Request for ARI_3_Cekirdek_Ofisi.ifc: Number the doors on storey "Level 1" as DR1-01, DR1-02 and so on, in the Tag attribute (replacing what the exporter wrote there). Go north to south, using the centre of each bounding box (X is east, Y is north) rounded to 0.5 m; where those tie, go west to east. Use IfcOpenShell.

First a look at what the model holds.

```python
import ifcopenshell
import ifcopenshell.util.element
import ifcopenshell.util.placement

model = ifcopenshell.open("ARI_3_Cekirdek_Ofisi.ifc")
print(model.schema)
storey = next(s for s in model.by_type("IfcBuildingStorey") if s.Name == "Level 1")
doors = [e for e in ifcopenshell.util.element.get_decomposition(storey) if e.is_a("IfcDoor")]
for e in sorted(doors, key=lambda e: e.id()):
    origin = ifcopenshell.util.placement.get_local_placement(e.ObjectPlacement)[:3, 3]
    print(e.id(), e.Tag, e.Name, origin.round(2) + 0.0, sep=" | ")
```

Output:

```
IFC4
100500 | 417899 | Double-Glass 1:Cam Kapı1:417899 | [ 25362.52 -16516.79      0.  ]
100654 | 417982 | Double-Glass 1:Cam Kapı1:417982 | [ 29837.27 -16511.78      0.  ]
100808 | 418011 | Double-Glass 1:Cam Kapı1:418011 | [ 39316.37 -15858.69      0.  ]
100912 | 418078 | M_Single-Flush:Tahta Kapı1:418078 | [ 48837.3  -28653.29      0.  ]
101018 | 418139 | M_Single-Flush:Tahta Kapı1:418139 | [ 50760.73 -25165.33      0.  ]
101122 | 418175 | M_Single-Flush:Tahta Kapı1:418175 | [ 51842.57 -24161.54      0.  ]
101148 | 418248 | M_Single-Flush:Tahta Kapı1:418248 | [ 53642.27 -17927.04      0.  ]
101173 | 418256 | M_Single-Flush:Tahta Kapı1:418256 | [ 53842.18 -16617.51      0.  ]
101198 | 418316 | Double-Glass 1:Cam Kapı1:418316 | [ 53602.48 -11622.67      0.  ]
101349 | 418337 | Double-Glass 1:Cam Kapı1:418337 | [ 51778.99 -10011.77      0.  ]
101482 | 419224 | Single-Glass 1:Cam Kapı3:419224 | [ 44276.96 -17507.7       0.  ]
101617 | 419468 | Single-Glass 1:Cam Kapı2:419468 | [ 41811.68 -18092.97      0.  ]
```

```python
import ifcopenshell
import ifcopenshell.geom
import ifcopenshell.util.element
import ifcopenshell.util.shape

model = ifcopenshell.open("ARI_3_Cekirdek_Ofisi.ifc")
settings = ifcopenshell.geom.settings()
settings.set("use-world-coords", True)


def centre(element):
    shape = ifcopenshell.geom.create_shape(settings, element)
    return ifcopenshell.util.shape.get_bbox_centroid(shape.geometry)


storey = next(s for s in model.by_type("IfcBuildingStorey") if s.Name == "Level 1")
doors = [e for e in ifcopenshell.util.element.get_decomposition(storey) if e.is_a("IfcDoor")]

# Insertion points can sit at a corner or the storey origin, so sort by the geometry (in metres).
centres = {e: centre(e) for e in doors}
doors.sort(key=lambda e: (-round(centres[e][1] / 0.5), centres[e][0]))

for i, e in enumerate(doors, start=1):
    number = f"DR1-{i:02d}"
    e.Tag = number
    print(e.id(), number)

model.write("ARI_3_Cekirdek_Ofisi_edited.ifc")
```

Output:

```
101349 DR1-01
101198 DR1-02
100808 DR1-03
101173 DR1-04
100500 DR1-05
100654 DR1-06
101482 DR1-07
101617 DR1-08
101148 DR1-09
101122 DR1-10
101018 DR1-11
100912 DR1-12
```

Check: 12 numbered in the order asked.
